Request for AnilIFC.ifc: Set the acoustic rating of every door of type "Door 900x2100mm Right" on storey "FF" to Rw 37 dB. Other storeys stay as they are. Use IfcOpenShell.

First a look at what the model holds.

```python
import ifcopenshell
import ifcopenshell.util.element

model = ifcopenshell.open("AnilIFC.ifc")
print(model.schema)
storey = next(s for s in model.by_type("IfcBuildingStorey") if s.Name == "FF")
doors = [e for e in ifcopenshell.util.element.get_decomposition(storey) if e.is_a("IfcDoor")]
seen = {}
for e in doors:
    element_type = ifcopenshell.util.element.get_type(e)
    key = (element_type.Name if element_type != e and element_type else None, ifcopenshell.util.element.get_pset(e, "Pset_DoorCommon", "AcousticRating"))
    seen[key] = seen.get(key, 0) + 1
for (name, value), count in sorted(seen.items(), key=str):
    print(count, "x", name, "|", value)
```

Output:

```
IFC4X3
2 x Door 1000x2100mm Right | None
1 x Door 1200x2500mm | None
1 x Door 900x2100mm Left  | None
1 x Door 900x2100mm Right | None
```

```python
import ifcopenshell
import ifcopenshell.api.pset
import ifcopenshell.util.element

model = ifcopenshell.open("AnilIFC.ifc")

storey = next(s for s in model.by_type("IfcBuildingStorey") if s.Name == "FF")
doors = [e for e in ifcopenshell.util.element.get_decomposition(storey) if e.is_a("IfcDoor")]

count = 0
for e in doors:
    element_type = ifcopenshell.util.element.get_type(e)
    if element_type in (None, e) or element_type.Name != "Door 900x2100mm Right":
        continue
    # add_pset returns the element's existing set when there is one.
    pset = ifcopenshell.api.pset.add_pset(model, product=e, name="Pset_DoorCommon")
    ifcopenshell.api.pset.edit_pset(model, pset=pset, properties={"AcousticRating": "Rw 37 dB"})
    count += 1

print(count, "doors updated")

model.write("AnilIFC_v2.ifc")
```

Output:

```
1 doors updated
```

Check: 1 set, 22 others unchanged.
